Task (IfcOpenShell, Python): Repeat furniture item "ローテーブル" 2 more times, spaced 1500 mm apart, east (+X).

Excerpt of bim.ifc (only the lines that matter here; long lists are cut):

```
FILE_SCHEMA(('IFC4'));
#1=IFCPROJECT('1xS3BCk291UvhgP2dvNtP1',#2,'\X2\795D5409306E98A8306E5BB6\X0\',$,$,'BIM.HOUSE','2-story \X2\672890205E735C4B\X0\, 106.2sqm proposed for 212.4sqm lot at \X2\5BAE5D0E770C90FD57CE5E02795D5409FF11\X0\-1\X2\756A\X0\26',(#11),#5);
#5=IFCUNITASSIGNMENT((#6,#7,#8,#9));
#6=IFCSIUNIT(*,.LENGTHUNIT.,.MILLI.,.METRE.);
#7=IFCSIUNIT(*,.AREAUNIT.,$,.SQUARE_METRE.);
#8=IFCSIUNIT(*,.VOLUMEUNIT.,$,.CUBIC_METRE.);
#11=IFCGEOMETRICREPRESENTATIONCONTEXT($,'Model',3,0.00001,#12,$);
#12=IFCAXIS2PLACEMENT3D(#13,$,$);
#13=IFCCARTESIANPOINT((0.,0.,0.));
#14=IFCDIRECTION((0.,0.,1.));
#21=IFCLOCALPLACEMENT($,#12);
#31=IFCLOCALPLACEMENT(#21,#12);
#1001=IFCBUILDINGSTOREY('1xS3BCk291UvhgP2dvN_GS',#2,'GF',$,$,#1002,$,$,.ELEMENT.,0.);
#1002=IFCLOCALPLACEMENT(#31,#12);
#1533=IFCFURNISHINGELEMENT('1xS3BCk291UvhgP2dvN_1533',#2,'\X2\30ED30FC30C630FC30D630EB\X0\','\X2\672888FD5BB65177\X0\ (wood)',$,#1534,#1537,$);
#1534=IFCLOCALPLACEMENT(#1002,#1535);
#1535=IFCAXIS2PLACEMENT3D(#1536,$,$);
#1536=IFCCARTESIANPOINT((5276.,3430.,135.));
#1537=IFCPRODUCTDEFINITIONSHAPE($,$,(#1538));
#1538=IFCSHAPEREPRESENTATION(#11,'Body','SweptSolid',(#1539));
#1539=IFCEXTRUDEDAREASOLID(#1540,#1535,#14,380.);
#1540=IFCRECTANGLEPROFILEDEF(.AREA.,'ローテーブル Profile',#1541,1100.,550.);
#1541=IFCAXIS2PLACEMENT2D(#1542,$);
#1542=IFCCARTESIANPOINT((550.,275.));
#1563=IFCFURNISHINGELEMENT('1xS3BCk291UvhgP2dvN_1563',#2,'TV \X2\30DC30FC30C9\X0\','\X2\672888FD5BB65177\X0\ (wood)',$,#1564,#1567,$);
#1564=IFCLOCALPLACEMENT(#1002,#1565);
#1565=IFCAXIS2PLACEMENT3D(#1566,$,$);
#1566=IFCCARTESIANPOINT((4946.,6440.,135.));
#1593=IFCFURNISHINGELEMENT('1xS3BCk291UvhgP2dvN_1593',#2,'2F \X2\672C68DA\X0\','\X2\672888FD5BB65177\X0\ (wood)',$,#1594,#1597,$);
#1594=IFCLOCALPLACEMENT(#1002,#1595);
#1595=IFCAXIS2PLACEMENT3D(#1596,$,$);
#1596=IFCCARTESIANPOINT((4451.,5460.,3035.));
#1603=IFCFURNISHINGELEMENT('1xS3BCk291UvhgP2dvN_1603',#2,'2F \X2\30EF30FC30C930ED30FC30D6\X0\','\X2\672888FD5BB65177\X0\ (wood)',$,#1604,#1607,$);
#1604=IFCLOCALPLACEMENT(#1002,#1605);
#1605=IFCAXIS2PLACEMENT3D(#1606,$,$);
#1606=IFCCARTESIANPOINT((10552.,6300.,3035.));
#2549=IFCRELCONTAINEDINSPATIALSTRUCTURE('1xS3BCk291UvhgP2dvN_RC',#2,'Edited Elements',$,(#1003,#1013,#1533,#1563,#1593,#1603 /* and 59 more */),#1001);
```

```python
import numpy as np
import ifcopenshell
import ifcopenshell.api.geometry
import ifcopenshell.api.root
import ifcopenshell.util.element
import ifcopenshell.util.placement
import ifcopenshell.util.unit

model = ifcopenshell.open("bim.ifc")
unit_scale = ifcopenshell.util.unit.calculate_unit_scale(model)


def reuse_history(source, copy):
    """copy_class also copies each property set's owner history, people and application; keep the originals."""
    for rel in copy.IsDefinedBy:
        if rel.is_a("IfcRelDefinesByProperties") and (history := rel.RelatingPropertyDefinition.OwnerHistory):
            rel.RelatingPropertyDefinition.OwnerHistory = source.OwnerHistory
            ifcopenshell.util.element.remove_deep2(model, history)


source = model.by_guid("1xS3BCk291UvhgP2dvN_1533")
base = ifcopenshell.util.placement.get_local_placement(source.ObjectPlacement)
step = np.array([1.0, 0.0, 0.0]) * 1.5 / unit_scale

for i in range(1, 3):
    copy = ifcopenshell.api.root.copy_class(model, product=source)
    copy.Representation = ifcopenshell.util.element.copy_deep(
        model, source.Representation, exclude=["IfcGeometricRepresentationContext", "IfcRepresentationMap"]
    )
    reuse_history(source, copy)
    matrix = base.copy()
    matrix[:3, 3] += i * step
    print("added at", matrix[:3, 3].round(3) + 0.0)
    ifcopenshell.api.geometry.edit_object_placement(model, product=copy, matrix=matrix, is_si=False)

model.write("bim_rev.ifc")
```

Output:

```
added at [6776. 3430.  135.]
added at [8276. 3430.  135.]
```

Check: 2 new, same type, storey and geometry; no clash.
